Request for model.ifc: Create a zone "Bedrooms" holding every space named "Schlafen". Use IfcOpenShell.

First a look at what the model holds.

```python
import ifcopenshell

model = ifcopenshell.open("model.ifc")
print(model.schema)
seen = {}
for space in model.by_type("IfcSpace"):
    seen[space.Name] = seen.get(space.Name, 0) + 1
for name, count in sorted(seen.items(), key=str):
    print(count, "x", name)
print("zones:", [z.Name for z in model.by_type("IfcZone")][:20])
```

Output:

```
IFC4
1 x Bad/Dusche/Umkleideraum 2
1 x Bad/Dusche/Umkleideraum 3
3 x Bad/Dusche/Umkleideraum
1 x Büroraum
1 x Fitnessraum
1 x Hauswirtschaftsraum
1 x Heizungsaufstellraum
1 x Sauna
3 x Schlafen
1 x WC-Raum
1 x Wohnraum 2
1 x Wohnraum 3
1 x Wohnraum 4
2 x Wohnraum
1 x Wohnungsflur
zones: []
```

```python
import ifcopenshell
import ifcopenshell.api.group
import ifcopenshell.api.root

model = ifcopenshell.open("model.ifc")

names = {"Schlafen"}
spaces = [s for s in model.by_type("IfcSpace") if s.Name in names]

zone = ifcopenshell.api.root.create_entity(model, ifc_class="IfcZone", name="Bedrooms")
ifcopenshell.api.group.assign_group(model, products=spaces, group=zone)
print(len(spaces), "spaces in", zone.Name)

model.write("model_edited.ifc")
```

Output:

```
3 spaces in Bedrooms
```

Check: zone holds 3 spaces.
